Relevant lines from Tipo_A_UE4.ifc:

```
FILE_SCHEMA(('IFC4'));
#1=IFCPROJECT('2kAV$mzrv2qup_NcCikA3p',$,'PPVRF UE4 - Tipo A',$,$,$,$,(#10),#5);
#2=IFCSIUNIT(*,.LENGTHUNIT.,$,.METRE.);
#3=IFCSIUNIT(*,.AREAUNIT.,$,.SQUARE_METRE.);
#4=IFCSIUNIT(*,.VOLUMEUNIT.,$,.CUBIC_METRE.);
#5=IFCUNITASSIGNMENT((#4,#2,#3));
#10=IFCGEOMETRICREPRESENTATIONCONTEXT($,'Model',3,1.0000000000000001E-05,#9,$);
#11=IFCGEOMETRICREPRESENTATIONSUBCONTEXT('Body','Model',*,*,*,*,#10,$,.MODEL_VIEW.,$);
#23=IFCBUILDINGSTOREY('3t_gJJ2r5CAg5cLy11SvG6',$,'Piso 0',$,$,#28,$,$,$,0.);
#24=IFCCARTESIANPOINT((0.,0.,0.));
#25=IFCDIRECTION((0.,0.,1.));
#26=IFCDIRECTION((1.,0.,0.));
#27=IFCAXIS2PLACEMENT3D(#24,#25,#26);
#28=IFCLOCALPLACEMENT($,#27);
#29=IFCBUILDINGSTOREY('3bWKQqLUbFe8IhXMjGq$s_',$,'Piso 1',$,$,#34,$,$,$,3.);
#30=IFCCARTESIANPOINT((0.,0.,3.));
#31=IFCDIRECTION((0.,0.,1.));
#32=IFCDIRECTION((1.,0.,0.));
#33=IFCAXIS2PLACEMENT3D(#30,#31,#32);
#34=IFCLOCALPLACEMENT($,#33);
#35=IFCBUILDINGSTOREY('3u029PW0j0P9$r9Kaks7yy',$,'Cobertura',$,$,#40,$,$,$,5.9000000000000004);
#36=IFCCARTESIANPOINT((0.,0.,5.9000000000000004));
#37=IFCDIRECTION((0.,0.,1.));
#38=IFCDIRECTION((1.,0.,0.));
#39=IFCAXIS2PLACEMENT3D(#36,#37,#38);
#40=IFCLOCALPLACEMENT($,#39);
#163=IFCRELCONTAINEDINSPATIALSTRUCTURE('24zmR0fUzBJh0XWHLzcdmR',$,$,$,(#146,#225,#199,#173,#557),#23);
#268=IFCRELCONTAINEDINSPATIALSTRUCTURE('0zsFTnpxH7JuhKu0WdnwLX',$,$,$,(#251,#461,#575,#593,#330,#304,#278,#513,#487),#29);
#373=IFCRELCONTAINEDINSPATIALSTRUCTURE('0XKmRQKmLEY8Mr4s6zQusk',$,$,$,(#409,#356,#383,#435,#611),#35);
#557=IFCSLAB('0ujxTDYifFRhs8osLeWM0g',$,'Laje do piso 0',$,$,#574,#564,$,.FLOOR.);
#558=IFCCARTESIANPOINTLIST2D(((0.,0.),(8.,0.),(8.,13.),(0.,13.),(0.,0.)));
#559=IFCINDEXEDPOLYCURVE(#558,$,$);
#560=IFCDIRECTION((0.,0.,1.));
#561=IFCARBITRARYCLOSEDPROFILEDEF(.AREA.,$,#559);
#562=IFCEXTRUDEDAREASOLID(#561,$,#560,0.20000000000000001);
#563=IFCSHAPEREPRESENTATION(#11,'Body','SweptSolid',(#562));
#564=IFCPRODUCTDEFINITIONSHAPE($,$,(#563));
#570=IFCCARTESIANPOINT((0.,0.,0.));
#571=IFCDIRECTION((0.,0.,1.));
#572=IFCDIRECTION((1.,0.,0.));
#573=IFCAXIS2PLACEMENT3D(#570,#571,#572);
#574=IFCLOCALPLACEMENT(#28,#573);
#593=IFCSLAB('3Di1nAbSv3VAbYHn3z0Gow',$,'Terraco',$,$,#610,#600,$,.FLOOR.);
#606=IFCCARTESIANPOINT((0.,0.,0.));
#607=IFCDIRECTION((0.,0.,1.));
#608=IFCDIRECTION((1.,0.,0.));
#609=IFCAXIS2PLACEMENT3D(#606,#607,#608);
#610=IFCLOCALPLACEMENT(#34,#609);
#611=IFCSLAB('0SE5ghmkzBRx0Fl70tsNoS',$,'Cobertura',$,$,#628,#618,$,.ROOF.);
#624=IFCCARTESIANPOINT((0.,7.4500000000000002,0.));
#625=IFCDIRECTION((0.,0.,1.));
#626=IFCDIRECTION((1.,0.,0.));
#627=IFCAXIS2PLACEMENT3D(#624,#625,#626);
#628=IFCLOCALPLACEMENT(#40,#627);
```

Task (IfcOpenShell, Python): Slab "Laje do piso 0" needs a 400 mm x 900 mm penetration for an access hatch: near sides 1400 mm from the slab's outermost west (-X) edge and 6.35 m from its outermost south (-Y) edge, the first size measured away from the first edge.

```python
import numpy as np
import ifcopenshell
import ifcopenshell.api.feature
import ifcopenshell.api.geometry
import ifcopenshell.api.root
import ifcopenshell.geom
import ifcopenshell.util.placement
import ifcopenshell.util.representation
import ifcopenshell.util.shape
import ifcopenshell.util.unit

model = ifcopenshell.open("Tipo_A_UE4.ifc")
unit_scale = ifcopenshell.util.unit.calculate_unit_scale(model)
settings = ifcopenshell.geom.settings()


def volume(element):
    """Net volume in cubic metres, openings subtracted."""
    shape = ifcopenshell.geom.create_shape(settings, element)
    return ifcopenshell.util.shape.get_volume(shape.geometry)


slab = model.by_id(557)
before = volume(slab)

# Extent in the slab's own axes, in metres. The edges named are its -X and -Y sides.
slab_shape = ifcopenshell.geom.create_shape(settings, slab)
vertices = ifcopenshell.util.shape.get_vertices(slab_shape.geometry)
x_min, y_min, bottom = vertices.min(axis=0)
top = vertices[:, 2].max()

opening = ifcopenshell.api.root.create_entity(model, ifc_class="IfcOpeningElement", name="Access hatch opening", predefined_type="OPENING")
context = ifcopenshell.util.representation.get_context(model, "Model", "Body", "MODEL_VIEW")
width, depth = 0.4, 0.9
outline = [(0.0, 0.0), (width, 0.0), (width, depth), (0.0, depth), (0.0, 0.0)]
# Overshoot both faces by 50 mm so the cut is clean.
shape = ifcopenshell.api.geometry.add_slab_representation(
    model, context=context, depth=top - bottom + 0.1, polyline=outline
)
ifcopenshell.api.geometry.assign_representation(model, product=opening, representation=shape)

matrix = ifcopenshell.util.placement.get_local_placement(slab.ObjectPlacement)
matrix[:, 3] = matrix @ np.append(np.array([x_min + 1.4, y_min + 6.35, bottom - 0.05]) / unit_scale, 1.0)
ifcopenshell.api.geometry.edit_object_placement(model, product=opening, matrix=matrix, is_si=False)
ifcopenshell.api.feature.add_feature(model, feature=opening, element=slab)

after = volume(slab)

print(f"slab volume {before:.3f} -> {after:.3f} m3")

model.write("Tipo_A_UE4_updated.ifc")
```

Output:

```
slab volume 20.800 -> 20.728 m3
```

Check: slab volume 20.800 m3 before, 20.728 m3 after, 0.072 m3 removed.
